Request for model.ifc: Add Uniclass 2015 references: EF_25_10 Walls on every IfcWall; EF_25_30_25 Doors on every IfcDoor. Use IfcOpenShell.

First a look at what the model holds.

```python
import ifcopenshell

model = ifcopenshell.open("model.ifc")
print(model.schema)
print("classifications:", [c.Name for c in model.by_type("IfcClassification")])
for ifc_class in ("IfcDoor", "IfcRoof", "IfcStair", "IfcWall", "IfcWindow"):
    print(ifc_class, len(model.by_type(ifc_class)))
```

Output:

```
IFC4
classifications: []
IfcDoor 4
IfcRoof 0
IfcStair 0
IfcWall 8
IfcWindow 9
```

```python
import ifcopenshell
import ifcopenshell.api.classification

model = ifcopenshell.open("model.ifc")

system = ifcopenshell.api.classification.add_classification(model, classification="Uniclass 2015")

codes = {
    "IfcWall": ("EF_25_10", "Walls"),
    "IfcDoor": ("EF_25_30_25", "Doors"),
}
for ifc_class, (code, name) in codes.items():
    products = model.by_type(ifc_class)
    ifcopenshell.api.classification.add_reference(
        model, products=products, classification=system, identification=code, name=name
    )
    print(code, len(products))

model.write("model_rev.ifc")
```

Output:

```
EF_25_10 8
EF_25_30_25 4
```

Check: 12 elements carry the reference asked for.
